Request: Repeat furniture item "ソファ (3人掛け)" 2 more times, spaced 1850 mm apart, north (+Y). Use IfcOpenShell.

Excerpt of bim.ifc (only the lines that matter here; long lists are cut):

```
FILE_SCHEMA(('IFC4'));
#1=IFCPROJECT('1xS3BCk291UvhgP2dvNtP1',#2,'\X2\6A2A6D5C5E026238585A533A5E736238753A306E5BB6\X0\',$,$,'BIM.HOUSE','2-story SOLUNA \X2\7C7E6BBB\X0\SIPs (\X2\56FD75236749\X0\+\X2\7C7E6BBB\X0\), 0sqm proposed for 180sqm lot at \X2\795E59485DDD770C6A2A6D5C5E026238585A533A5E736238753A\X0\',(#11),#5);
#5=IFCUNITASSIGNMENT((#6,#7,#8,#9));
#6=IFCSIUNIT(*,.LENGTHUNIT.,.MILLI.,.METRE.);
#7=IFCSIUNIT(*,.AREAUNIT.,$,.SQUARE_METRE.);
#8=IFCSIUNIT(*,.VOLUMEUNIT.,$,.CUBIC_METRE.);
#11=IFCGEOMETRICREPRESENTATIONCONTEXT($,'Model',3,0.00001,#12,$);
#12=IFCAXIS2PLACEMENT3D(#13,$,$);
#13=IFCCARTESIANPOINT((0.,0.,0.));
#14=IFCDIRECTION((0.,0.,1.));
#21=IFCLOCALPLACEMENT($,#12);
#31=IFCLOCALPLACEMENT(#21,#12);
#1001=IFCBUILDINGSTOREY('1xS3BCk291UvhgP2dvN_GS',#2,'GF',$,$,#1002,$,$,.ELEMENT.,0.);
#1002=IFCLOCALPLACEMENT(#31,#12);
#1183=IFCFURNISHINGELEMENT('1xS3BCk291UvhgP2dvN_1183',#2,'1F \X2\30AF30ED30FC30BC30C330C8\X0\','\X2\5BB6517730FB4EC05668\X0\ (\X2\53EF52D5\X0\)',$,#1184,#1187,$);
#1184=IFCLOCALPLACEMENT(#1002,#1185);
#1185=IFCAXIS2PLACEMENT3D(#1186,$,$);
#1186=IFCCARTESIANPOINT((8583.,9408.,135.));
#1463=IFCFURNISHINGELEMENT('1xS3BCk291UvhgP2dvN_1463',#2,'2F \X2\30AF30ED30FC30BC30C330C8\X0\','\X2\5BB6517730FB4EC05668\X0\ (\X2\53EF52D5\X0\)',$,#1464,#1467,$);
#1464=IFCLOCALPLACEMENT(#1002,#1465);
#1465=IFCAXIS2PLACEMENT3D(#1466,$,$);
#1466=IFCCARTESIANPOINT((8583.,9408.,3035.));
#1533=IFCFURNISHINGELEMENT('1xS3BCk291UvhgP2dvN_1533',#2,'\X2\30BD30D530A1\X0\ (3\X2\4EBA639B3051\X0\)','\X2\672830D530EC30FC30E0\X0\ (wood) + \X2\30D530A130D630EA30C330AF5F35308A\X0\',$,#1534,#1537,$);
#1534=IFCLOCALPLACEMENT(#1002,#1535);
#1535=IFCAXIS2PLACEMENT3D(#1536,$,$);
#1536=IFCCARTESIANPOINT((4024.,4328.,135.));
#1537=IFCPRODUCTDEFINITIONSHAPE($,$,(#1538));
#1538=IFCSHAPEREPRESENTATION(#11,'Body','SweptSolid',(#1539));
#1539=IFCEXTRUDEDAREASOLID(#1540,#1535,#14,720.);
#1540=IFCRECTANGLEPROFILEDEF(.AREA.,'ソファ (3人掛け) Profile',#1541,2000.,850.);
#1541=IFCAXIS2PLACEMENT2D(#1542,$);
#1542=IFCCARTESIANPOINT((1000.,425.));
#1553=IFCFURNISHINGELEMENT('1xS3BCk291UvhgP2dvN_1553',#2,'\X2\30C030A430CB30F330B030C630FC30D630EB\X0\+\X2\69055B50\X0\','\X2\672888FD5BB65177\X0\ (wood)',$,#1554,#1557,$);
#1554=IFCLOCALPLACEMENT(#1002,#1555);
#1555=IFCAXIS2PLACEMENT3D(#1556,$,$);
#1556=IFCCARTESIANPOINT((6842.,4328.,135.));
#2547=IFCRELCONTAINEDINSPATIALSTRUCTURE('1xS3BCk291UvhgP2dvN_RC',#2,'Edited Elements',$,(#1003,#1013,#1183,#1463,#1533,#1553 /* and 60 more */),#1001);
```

```python
import numpy as np
import ifcopenshell
import ifcopenshell.api.geometry
import ifcopenshell.api.root
import ifcopenshell.util.element
import ifcopenshell.util.placement

model = ifcopenshell.open("bim.ifc")


def reuse_history(source, copy):
    """copy_class also copies each property set's owner history, people and application; keep the originals."""
    for rel in copy.IsDefinedBy:
        if rel.is_a("IfcRelDefinesByProperties") and (history := rel.RelatingPropertyDefinition.OwnerHistory):
            rel.RelatingPropertyDefinition.OwnerHistory = source.OwnerHistory
            ifcopenshell.util.element.remove_deep2(model, history)


source = model.by_guid("1xS3BCk291UvhgP2dvN_1533")
base = ifcopenshell.util.placement.get_local_placement(source.ObjectPlacement)
step = np.array([0.0, 1.0, 0.0]) * 1850.0

for i in range(1, 3):
    copy = ifcopenshell.api.root.copy_class(model, product=source)
    copy.Representation = ifcopenshell.util.element.copy_deep(
        model, source.Representation, exclude=["IfcGeometricRepresentationContext", "IfcRepresentationMap"]
    )
    reuse_history(source, copy)
    matrix = base.copy()
    matrix[:3, 3] += i * step
    print("added at", matrix[:3, 3].round(3) + 0.0)
    ifcopenshell.api.geometry.edit_object_placement(model, product=copy, matrix=matrix, is_si=False)

model.write("bim_edited.ifc")
```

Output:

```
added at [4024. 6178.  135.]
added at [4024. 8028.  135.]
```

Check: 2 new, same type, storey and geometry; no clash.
